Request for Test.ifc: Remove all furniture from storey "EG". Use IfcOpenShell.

First a look at what the model holds.

```python
import ifcopenshell
import ifcopenshell.util.element

model = ifcopenshell.open("Test.ifc")
print(model.schema)
storey = next(s for s in model.by_type("IfcBuildingStorey") if s.Name == "EG")
furniture = [e for e in ifcopenshell.util.element.get_decomposition(storey) if e.is_a("IfcFurnishingElement")]
seen = {}
for e in furniture:
    element_type = ifcopenshell.util.element.get_type(e)
    name = element_type.Name if element_type not in (None, e) else None
    seen[name] = seen.get(name, 0) + 1
for name, count in sorted(seen.items(), key=str):
    print(count, "x", name)
```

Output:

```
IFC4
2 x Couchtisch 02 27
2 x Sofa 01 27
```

```python
import ifcopenshell
import ifcopenshell.api.root
import ifcopenshell.util.element

model = ifcopenshell.open("Test.ifc")

storey = next(s for s in model.by_type("IfcBuildingStorey") if s.Name == "EG")
furniture = [e for e in ifcopenshell.util.element.get_decomposition(storey) if e.is_a("IfcFurnishingElement")]

for e in furniture:
    ifcopenshell.api.root.remove_product(model, product=e)
print(len(furniture), "removed")

model.write("Test_v2.ifc")
```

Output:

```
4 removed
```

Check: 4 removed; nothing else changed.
